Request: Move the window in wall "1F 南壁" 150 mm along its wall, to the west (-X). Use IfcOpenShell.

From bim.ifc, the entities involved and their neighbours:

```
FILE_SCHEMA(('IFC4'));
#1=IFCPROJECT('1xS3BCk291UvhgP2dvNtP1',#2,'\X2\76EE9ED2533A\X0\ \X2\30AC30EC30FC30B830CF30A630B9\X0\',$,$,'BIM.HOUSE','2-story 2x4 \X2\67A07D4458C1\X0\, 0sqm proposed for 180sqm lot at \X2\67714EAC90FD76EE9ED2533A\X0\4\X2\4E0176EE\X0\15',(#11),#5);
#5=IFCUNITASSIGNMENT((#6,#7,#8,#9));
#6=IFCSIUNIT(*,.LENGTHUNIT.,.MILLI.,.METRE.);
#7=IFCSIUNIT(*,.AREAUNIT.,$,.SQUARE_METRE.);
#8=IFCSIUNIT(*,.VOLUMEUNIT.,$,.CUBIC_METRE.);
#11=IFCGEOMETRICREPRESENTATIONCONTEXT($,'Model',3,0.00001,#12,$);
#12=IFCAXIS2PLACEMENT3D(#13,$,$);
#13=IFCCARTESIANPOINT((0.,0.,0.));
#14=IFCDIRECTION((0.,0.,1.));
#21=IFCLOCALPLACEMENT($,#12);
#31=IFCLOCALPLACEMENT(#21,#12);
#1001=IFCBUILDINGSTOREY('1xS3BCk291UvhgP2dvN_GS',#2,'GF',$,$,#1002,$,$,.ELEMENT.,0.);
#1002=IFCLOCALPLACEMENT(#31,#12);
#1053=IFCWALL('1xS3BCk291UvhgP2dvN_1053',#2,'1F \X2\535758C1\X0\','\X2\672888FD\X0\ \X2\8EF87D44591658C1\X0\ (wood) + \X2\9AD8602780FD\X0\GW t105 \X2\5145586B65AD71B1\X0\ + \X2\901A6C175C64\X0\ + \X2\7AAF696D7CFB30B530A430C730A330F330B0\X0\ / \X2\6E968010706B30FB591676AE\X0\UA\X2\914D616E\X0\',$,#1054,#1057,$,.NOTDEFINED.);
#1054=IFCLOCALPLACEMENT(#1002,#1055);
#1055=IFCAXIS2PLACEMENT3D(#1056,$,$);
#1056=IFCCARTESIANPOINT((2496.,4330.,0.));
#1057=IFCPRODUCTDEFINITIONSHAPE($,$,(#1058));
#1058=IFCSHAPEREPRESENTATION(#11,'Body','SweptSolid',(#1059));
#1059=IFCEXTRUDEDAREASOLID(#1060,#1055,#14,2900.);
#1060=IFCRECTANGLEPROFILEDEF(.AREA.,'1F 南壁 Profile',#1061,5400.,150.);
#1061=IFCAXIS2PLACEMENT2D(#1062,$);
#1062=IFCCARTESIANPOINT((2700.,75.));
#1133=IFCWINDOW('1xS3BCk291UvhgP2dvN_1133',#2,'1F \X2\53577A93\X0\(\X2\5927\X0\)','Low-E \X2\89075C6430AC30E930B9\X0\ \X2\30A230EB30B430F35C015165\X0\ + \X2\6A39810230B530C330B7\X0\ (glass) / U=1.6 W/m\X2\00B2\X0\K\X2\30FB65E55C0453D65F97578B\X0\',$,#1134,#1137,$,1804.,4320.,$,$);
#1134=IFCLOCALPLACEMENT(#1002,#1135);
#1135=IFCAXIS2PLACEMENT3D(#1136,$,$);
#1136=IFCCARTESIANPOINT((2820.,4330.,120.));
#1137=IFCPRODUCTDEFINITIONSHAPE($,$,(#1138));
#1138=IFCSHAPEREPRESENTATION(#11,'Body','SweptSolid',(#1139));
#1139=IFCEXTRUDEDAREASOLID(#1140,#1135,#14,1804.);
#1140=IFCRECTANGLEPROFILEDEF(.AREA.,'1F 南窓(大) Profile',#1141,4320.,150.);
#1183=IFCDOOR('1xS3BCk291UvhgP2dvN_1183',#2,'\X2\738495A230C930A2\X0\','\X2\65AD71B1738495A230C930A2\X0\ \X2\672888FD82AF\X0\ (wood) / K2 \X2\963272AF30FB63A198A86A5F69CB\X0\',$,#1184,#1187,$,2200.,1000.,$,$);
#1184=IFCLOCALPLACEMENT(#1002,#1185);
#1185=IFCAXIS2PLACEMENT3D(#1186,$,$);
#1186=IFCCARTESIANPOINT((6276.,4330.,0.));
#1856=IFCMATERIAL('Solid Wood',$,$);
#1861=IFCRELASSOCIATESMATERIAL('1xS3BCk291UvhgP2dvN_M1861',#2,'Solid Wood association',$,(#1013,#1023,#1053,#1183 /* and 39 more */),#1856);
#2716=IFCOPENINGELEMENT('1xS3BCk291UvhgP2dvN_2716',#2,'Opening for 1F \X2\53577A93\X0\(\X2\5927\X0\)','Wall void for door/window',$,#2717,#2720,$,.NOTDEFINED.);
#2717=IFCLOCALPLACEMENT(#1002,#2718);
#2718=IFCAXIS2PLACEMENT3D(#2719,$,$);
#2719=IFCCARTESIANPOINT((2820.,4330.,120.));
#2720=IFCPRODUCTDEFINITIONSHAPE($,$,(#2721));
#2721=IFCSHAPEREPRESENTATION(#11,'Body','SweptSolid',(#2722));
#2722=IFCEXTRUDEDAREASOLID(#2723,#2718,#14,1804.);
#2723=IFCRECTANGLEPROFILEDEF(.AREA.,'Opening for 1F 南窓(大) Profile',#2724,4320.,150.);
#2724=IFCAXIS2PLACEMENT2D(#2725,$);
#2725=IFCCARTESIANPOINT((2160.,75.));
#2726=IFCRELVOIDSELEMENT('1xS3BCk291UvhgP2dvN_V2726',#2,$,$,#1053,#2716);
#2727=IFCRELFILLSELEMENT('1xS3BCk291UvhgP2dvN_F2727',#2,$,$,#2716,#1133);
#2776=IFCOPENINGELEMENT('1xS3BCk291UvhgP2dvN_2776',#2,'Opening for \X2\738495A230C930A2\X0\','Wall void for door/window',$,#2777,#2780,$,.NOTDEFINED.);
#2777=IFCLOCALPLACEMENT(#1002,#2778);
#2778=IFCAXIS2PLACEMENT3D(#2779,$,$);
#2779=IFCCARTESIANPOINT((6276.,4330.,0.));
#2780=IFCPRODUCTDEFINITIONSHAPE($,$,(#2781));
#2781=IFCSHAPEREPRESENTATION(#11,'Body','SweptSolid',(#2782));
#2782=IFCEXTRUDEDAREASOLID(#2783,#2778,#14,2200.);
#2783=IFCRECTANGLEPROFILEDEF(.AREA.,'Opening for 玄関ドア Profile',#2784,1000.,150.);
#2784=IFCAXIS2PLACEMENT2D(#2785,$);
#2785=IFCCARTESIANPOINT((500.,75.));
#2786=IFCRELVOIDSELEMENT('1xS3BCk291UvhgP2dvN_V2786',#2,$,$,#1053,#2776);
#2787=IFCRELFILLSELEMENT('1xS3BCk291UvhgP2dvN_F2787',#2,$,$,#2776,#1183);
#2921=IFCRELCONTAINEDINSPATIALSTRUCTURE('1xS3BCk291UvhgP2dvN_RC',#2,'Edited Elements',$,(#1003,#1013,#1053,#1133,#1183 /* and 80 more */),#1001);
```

```python
import ifcopenshell
import ifcopenshell.api.geometry
import ifcopenshell.util.placement
import ifcopenshell.util.unit

model = ifcopenshell.open("bim.ifc")
unit_scale = ifcopenshell.util.unit.calculate_unit_scale(model)

window = model.by_guid("1xS3BCk291UvhgP2dvN_1133")
opening = window.FillsVoids[0].RelatingOpeningElement
wall = opening.VoidsElements[0].RelatingBuildingElement

wall_matrix = ifcopenshell.util.placement.get_local_placement(wall.ObjectPlacement)
shift = wall_matrix[:3, 0] * -0.15 / unit_scale
before = ifcopenshell.util.placement.get_local_placement(window.ObjectPlacement)[:3, 3].copy()

# The window is not placed relative to its opening, so move both.
for product in (opening, window):
    matrix = ifcopenshell.util.placement.get_local_placement(product.ObjectPlacement)
    matrix[:3, 3] += shift
    ifcopenshell.api.geometry.edit_object_placement(model, product=product, matrix=matrix, is_si=False)

after = ifcopenshell.util.placement.get_local_placement(window.ObjectPlacement)[:3, 3]
print("window moved by", (after - before).round(3) + 0.0)

model.write("bim_updated.ifc")
```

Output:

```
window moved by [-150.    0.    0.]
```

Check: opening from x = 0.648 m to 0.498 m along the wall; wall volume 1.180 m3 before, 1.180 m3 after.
